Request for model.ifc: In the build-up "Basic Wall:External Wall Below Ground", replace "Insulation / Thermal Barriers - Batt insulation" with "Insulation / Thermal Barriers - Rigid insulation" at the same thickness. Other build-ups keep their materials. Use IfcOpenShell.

First a look at what the model holds.

```python
import ifcopenshell
import ifcopenshell.util.element

model = ifcopenshell.open("model.ifc")
print(model.schema)
for layer_set in model.by_type("IfcMaterialLayerSet"):
    if layer_set.LayerSetName == "Basic Wall:External Wall Below Ground":
        for layer in layer_set.MaterialLayers:
            print(layer.id(), layer.Material and layer.Material.Name, layer.LayerThickness, sep=" | ")
        print(len(ifcopenshell.util.element.get_elements_by_material(model, layer_set)), "elements and types use it")
print(sorted(m.Name for m in model.by_type("IfcMaterial") if m.Name)[:60])
```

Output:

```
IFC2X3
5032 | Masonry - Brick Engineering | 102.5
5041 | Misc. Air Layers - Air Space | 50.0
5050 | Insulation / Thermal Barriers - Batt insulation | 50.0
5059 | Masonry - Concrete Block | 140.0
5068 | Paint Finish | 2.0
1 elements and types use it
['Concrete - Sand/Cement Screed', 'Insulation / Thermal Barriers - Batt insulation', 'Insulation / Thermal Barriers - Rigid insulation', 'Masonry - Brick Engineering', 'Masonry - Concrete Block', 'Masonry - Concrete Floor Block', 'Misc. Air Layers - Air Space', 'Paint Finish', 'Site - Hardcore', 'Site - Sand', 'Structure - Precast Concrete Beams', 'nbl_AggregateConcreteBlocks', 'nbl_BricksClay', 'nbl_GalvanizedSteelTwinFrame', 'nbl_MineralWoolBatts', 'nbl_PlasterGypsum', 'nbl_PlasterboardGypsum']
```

```python
import ifcopenshell
import ifcopenshell.api.material

model = ifcopenshell.open("model.ifc")

layer_set = next(s for s in model.by_type("IfcMaterialLayerSet") if s.LayerSetName == "Basic Wall:External Wall Below Ground")
layer = next(l for l in layer_set.MaterialLayers if l.Material and l.Material.Name == "Insulation / Thermal Barriers - Batt insulation")
material = next(m for m in model.by_type("IfcMaterial") if m.Name == "Insulation / Thermal Barriers - Rigid insulation")

# Point this one layer at the other material; renaming the old one would change it everywhere.
ifcopenshell.api.material.edit_layer(model, layer=layer, attributes={}, material=material)

print([l.Material.Name if l.Material else None for l in layer_set.MaterialLayers])

model.write("model_v2.ifc")
```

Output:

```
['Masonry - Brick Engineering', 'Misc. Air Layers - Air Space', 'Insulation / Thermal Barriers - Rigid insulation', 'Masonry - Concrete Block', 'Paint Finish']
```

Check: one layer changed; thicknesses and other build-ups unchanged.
